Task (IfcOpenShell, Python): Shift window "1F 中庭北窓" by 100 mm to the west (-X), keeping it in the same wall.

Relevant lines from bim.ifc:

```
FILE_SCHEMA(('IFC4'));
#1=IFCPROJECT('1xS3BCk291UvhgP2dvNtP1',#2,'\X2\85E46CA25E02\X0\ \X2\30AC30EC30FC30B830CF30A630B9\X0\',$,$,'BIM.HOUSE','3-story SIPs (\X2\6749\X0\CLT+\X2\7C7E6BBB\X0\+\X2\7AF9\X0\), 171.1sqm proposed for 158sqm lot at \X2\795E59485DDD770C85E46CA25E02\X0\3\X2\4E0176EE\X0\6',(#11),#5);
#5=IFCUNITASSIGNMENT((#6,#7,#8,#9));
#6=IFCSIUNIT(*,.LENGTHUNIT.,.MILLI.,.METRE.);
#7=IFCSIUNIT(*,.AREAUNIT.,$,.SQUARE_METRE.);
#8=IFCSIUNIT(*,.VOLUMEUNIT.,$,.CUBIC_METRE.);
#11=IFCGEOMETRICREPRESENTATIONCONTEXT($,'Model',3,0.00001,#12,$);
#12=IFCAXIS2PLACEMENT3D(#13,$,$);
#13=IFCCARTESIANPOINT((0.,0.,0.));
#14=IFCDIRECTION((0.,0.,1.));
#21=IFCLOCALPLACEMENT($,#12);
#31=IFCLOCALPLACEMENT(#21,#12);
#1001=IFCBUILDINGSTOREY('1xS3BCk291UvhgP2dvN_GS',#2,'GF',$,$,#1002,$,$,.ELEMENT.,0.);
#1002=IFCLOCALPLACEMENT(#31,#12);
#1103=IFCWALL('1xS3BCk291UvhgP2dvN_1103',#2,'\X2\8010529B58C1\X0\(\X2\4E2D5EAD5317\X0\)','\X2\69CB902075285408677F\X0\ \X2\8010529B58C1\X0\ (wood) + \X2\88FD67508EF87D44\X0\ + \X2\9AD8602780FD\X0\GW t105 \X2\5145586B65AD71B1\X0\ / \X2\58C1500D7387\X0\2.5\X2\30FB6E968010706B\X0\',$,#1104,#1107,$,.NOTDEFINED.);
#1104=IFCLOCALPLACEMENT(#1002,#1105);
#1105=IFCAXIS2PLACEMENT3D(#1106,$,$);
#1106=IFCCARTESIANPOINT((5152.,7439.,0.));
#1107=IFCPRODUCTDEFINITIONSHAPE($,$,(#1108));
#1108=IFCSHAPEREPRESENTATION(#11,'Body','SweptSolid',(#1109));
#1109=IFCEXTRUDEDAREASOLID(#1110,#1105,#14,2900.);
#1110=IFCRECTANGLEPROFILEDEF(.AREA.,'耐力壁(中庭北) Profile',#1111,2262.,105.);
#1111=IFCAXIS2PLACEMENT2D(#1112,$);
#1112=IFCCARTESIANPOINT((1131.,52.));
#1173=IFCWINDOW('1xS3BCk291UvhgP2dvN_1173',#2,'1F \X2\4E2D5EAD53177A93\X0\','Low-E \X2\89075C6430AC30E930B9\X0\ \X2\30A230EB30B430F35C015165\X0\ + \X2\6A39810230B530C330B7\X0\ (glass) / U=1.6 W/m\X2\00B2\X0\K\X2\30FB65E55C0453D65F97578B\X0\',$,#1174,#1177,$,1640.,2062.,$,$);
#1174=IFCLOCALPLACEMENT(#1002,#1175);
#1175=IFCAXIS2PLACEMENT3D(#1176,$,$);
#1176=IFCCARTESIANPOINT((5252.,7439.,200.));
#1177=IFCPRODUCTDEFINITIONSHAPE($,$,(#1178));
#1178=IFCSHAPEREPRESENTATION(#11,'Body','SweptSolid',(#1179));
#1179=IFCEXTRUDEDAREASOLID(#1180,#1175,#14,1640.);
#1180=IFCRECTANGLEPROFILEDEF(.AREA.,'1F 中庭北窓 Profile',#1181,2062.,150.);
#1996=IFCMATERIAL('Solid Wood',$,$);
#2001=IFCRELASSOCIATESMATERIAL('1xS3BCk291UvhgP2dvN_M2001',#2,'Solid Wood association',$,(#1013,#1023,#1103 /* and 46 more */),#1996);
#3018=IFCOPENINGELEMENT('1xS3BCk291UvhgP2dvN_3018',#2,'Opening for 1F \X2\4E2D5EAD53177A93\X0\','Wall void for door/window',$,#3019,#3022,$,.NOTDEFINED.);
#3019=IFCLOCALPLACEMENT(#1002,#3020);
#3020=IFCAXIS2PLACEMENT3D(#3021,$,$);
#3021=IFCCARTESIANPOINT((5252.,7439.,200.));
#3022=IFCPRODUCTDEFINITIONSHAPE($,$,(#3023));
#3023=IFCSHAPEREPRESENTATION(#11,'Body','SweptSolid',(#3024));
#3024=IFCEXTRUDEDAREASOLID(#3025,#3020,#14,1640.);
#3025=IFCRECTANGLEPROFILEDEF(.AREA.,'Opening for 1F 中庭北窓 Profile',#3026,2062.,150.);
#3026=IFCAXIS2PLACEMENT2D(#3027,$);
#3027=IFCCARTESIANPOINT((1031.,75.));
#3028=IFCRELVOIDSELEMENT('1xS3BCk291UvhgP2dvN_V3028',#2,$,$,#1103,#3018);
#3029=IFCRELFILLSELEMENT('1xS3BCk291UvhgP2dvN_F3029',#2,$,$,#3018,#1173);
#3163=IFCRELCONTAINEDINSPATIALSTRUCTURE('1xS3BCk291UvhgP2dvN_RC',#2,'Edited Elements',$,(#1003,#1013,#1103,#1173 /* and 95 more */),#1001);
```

```python
import ifcopenshell
import ifcopenshell.api.geometry
import ifcopenshell.util.placement
import ifcopenshell.util.unit

model = ifcopenshell.open("bim.ifc")
unit_scale = ifcopenshell.util.unit.calculate_unit_scale(model)

window = model.by_guid("1xS3BCk291UvhgP2dvN_1173")
opening = window.FillsVoids[0].RelatingOpeningElement
wall = opening.VoidsElements[0].RelatingBuildingElement

wall_matrix = ifcopenshell.util.placement.get_local_placement(wall.ObjectPlacement)
shift = wall_matrix[:3, 0] * -0.1 / unit_scale
before = ifcopenshell.util.placement.get_local_placement(window.ObjectPlacement)[:3, 3].copy()

# The window is not placed relative to its opening, so move both.
for product in (opening, window):
    matrix = ifcopenshell.util.placement.get_local_placement(product.ObjectPlacement)
    matrix[:3, 3] += shift
    ifcopenshell.api.geometry.edit_object_placement(model, product=product, matrix=matrix, is_si=False)

after = ifcopenshell.util.placement.get_local_placement(window.ObjectPlacement)[:3, 3]
print("window moved by", (after - before).round(3) + 0.0)

model.write("bim_edited.ifc")
```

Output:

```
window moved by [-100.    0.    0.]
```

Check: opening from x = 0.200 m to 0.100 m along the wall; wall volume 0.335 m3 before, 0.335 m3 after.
